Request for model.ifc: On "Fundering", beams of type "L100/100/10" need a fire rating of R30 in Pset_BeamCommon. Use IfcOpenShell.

First a look at what the model holds.

```python
import ifcopenshell
import ifcopenshell.util.element

model = ifcopenshell.open("model.ifc")
print(model.schema)
storey = next(s for s in model.by_type("IfcBuildingStorey") if s.Name == "Fundering")
beams = [e for e in ifcopenshell.util.element.get_decomposition(storey) if e.is_a("IfcBeam")]
seen = {}
for e in beams:
    element_type = ifcopenshell.util.element.get_type(e)
    key = (element_type.Name if element_type != e and element_type else None, ifcopenshell.util.element.get_pset(e, "Pset_BeamCommon", "FireRating"))
    seen[key] = seen.get(key, 0) + 1
for (name, value), count in sorted(seen.items(), key=str):
    print(count, "x", name, "|", value)
```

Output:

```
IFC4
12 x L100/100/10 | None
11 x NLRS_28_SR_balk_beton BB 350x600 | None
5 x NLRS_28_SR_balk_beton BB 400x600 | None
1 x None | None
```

```python
import ifcopenshell
import ifcopenshell.api.pset
import ifcopenshell.util.element

model = ifcopenshell.open("model.ifc")

storey = next(s for s in model.by_type("IfcBuildingStorey") if s.Name == "Fundering")
beams = [e for e in ifcopenshell.util.element.get_decomposition(storey) if e.is_a("IfcBeam")]

count = 0
for e in beams:
    element_type = ifcopenshell.util.element.get_type(e)
    if element_type in (None, e) or element_type.Name != "L100/100/10":
        continue
    # add_pset returns the element's existing set when there is one.
    pset = ifcopenshell.api.pset.add_pset(model, product=e, name="Pset_BeamCommon")
    ifcopenshell.api.pset.edit_pset(model, pset=pset, properties={"FireRating": "R30"})
    count += 1

print(count, "beams updated")

model.write("model-out.ifc")
```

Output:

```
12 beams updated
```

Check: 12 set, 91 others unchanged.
